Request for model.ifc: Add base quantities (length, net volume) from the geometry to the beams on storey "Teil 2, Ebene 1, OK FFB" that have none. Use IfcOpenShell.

First a look at what the model holds.

```python
import ifcopenshell
import ifcopenshell.util.element
import ifcopenshell.util.unit

model = ifcopenshell.open("model.ifc")
print(model.schema)
for unit_type in ("LENGTHUNIT", "AREAUNIT", "VOLUMEUNIT"):
    print(unit_type, ifcopenshell.util.unit.calculate_unit_scale(model, unit_type))
storey = next(s for s in model.by_type("IfcBuildingStorey") if s.Name == "Teil 2, Ebene 1, OK FFB")
beams = [e for e in ifcopenshell.util.element.get_decomposition(storey) if e.is_a("IfcBeam")]
for e in sorted(beams, key=lambda e: e.id()):
    print(e.id(), e.is_a(), e.Name, list(ifcopenshell.util.element.get_psets(e, qtos_only=True)), sep=" | ")
```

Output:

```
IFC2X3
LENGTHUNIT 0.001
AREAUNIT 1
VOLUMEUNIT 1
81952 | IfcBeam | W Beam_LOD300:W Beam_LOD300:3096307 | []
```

```python
import ifcopenshell
import ifcopenshell.api.pset
import ifcopenshell.geom
import ifcopenshell.util.element
import ifcopenshell.util.shape
import ifcopenshell.util.unit

model = ifcopenshell.open("model.ifc")
unit_scale = ifcopenshell.util.unit.calculate_unit_scale(model)
volume_scale = ifcopenshell.util.unit.calculate_unit_scale(model, "VOLUMEUNIT")
settings = ifcopenshell.geom.settings()

storey = next(s for s in model.by_type("IfcBuildingStorey") if s.Name == "Teil 2, Ebene 1, OK FFB")
beams = [e for e in ifcopenshell.util.element.get_decomposition(storey) if e.is_a("IfcBeam")]

for e in sorted(beams, key=lambda e: e.id()):
    if ifcopenshell.util.element.get_psets(e, qtos_only=True, should_inherit=False):
        continue
    # Geometry comes back in metres, in the element's own axes.
    shape = ifcopenshell.geom.create_shape(settings, e)
    values = {
        "Length": ifcopenshell.util.shape.get_max_xyz(shape.geometry) / unit_scale,
        "NetVolume": ifcopenshell.util.shape.get_volume(shape.geometry) / volume_scale,
    }
    qto = ifcopenshell.api.pset.add_qto(model, product=e, name="BaseQuantities")
    ifcopenshell.api.pset.edit_qto(model, qto=qto, properties=values)
    print(e.id(), {k: round(v, 3) for k, v in values.items()})

model.write("model-out.ifc")
```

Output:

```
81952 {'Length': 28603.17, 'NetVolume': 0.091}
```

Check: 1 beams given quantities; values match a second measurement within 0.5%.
